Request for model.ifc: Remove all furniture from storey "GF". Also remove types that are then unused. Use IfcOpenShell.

First a look at what the model holds.

```python
import ifcopenshell
import ifcopenshell.util.element

model = ifcopenshell.open("model.ifc")
print(model.schema)
storey = next(s for s in model.by_type("IfcBuildingStorey") if s.Name == "GF")
furniture = [e for e in ifcopenshell.util.element.get_decomposition(storey) if e.is_a("IfcFurnishingElement")]
seen = {}
for e in furniture:
    element_type = ifcopenshell.util.element.get_type(e)
    name = element_type.Name if element_type not in (None, e) else None
    seen[name] = seen.get(name, 0) + 1
for name, count in sorted(seen.items(), key=str):
    print(count, "x", name)
```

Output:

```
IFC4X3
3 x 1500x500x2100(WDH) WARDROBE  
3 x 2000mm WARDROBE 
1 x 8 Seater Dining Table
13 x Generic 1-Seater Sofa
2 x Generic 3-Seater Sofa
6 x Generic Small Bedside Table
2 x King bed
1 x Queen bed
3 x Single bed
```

```python
import ifcopenshell
import ifcopenshell.api.root
import ifcopenshell.util.element

model = ifcopenshell.open("model.ifc")

storey = next(s for s in model.by_type("IfcBuildingStorey") if s.Name == "GF")
furniture = [e for e in ifcopenshell.util.element.get_decomposition(storey) if e.is_a("IfcFurnishingElement")]
types = {ifcopenshell.util.element.get_type(e) for e in furniture} - {None, *furniture}

for e in furniture:
    ifcopenshell.api.root.remove_product(model, product=e)
print(len(furniture), "removed")

unused = [t for t in types if not ifcopenshell.util.element.get_types(t)]
for t in unused:
    ifcopenshell.api.root.remove_product(model, product=t)
print(len(unused), "unused types removed")

model.write("model_edited.ifc")
```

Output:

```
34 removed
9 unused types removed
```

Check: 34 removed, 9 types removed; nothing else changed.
